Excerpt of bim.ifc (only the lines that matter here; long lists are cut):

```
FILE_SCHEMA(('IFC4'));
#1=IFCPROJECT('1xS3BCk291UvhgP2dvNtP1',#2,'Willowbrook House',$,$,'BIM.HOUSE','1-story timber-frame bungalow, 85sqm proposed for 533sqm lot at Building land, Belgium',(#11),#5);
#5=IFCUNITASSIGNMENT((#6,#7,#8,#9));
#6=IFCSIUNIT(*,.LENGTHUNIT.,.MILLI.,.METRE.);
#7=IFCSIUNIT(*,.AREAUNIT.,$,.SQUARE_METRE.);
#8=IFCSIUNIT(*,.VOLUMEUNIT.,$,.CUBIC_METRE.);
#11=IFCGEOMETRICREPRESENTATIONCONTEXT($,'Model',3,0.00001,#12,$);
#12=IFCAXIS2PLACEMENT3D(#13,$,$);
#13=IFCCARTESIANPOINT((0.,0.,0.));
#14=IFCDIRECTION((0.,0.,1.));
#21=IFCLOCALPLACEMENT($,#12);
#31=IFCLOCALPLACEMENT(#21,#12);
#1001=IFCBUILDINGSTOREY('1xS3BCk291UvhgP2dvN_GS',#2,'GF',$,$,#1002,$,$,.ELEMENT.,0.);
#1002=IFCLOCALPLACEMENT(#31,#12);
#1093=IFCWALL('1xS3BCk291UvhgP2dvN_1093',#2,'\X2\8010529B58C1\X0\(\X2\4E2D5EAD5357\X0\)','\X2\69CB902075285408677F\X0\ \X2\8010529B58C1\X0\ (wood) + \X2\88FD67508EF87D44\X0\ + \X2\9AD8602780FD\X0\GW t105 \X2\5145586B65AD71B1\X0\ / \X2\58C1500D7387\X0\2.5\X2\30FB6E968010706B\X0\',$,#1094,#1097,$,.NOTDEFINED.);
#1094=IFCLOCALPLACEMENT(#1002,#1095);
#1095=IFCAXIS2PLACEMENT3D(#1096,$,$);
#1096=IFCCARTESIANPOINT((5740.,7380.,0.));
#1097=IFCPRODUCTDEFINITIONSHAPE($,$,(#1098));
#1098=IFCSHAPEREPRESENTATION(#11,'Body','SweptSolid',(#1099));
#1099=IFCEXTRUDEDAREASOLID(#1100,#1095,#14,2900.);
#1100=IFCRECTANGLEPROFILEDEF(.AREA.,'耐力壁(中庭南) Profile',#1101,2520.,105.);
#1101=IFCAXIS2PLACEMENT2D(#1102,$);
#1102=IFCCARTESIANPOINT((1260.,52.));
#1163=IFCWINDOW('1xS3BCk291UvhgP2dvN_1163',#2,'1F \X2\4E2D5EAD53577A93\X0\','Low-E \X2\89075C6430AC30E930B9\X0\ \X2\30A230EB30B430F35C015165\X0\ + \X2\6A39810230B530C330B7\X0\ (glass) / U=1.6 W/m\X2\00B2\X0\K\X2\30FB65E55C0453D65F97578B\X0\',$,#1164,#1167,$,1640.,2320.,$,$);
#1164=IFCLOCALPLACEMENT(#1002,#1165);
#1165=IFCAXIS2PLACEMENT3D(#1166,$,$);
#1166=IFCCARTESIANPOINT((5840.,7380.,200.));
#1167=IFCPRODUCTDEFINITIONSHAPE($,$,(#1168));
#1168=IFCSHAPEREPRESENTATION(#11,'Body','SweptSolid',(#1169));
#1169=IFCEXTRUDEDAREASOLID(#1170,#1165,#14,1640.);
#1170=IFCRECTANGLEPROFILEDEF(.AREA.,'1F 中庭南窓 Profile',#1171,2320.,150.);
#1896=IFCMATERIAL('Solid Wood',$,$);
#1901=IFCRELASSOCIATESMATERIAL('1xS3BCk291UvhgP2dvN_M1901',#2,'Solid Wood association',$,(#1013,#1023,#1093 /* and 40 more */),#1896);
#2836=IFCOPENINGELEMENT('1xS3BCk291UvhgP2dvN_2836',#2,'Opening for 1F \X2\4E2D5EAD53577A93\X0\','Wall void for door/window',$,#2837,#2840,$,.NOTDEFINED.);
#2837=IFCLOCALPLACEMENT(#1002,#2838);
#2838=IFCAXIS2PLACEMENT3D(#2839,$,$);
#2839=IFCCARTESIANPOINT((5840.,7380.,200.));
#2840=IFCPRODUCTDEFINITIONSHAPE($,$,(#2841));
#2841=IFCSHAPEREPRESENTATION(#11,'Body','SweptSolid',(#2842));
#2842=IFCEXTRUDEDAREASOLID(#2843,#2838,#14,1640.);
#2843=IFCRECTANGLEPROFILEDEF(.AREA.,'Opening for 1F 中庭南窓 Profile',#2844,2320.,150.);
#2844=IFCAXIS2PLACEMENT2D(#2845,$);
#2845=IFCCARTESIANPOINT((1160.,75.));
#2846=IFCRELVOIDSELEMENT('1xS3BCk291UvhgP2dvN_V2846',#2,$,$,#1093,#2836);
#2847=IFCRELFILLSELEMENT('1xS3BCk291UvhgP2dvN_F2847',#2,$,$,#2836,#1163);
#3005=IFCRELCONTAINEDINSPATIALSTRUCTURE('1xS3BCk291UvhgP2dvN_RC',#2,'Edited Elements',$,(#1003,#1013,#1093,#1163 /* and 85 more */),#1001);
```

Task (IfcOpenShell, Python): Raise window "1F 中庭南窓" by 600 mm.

```python
import numpy as np
import ifcopenshell
import ifcopenshell.api.geometry
import ifcopenshell.util.placement
import ifcopenshell.util.unit

model = ifcopenshell.open("bim.ifc")
unit_scale = ifcopenshell.util.unit.calculate_unit_scale(model)

window = model.by_guid("1xS3BCk291UvhgP2dvN_1163")
opening = window.FillsVoids[0].RelatingOpeningElement
dz = 600.0

shift = np.array([0.0, 0.0, dz])
# The window is not placed relative to its opening, so move both.
for product in (opening, window):
    matrix = ifcopenshell.util.placement.get_local_placement(product.ObjectPlacement)
    matrix[:3, 3] += shift
    ifcopenshell.api.geometry.edit_object_placement(model, product=product, matrix=matrix, is_si=False)

print(f"moved by {dz * unit_scale:+.3f} m")

model.write("bim_rev.ifc")
```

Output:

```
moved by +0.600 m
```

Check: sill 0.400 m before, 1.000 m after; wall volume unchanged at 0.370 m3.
